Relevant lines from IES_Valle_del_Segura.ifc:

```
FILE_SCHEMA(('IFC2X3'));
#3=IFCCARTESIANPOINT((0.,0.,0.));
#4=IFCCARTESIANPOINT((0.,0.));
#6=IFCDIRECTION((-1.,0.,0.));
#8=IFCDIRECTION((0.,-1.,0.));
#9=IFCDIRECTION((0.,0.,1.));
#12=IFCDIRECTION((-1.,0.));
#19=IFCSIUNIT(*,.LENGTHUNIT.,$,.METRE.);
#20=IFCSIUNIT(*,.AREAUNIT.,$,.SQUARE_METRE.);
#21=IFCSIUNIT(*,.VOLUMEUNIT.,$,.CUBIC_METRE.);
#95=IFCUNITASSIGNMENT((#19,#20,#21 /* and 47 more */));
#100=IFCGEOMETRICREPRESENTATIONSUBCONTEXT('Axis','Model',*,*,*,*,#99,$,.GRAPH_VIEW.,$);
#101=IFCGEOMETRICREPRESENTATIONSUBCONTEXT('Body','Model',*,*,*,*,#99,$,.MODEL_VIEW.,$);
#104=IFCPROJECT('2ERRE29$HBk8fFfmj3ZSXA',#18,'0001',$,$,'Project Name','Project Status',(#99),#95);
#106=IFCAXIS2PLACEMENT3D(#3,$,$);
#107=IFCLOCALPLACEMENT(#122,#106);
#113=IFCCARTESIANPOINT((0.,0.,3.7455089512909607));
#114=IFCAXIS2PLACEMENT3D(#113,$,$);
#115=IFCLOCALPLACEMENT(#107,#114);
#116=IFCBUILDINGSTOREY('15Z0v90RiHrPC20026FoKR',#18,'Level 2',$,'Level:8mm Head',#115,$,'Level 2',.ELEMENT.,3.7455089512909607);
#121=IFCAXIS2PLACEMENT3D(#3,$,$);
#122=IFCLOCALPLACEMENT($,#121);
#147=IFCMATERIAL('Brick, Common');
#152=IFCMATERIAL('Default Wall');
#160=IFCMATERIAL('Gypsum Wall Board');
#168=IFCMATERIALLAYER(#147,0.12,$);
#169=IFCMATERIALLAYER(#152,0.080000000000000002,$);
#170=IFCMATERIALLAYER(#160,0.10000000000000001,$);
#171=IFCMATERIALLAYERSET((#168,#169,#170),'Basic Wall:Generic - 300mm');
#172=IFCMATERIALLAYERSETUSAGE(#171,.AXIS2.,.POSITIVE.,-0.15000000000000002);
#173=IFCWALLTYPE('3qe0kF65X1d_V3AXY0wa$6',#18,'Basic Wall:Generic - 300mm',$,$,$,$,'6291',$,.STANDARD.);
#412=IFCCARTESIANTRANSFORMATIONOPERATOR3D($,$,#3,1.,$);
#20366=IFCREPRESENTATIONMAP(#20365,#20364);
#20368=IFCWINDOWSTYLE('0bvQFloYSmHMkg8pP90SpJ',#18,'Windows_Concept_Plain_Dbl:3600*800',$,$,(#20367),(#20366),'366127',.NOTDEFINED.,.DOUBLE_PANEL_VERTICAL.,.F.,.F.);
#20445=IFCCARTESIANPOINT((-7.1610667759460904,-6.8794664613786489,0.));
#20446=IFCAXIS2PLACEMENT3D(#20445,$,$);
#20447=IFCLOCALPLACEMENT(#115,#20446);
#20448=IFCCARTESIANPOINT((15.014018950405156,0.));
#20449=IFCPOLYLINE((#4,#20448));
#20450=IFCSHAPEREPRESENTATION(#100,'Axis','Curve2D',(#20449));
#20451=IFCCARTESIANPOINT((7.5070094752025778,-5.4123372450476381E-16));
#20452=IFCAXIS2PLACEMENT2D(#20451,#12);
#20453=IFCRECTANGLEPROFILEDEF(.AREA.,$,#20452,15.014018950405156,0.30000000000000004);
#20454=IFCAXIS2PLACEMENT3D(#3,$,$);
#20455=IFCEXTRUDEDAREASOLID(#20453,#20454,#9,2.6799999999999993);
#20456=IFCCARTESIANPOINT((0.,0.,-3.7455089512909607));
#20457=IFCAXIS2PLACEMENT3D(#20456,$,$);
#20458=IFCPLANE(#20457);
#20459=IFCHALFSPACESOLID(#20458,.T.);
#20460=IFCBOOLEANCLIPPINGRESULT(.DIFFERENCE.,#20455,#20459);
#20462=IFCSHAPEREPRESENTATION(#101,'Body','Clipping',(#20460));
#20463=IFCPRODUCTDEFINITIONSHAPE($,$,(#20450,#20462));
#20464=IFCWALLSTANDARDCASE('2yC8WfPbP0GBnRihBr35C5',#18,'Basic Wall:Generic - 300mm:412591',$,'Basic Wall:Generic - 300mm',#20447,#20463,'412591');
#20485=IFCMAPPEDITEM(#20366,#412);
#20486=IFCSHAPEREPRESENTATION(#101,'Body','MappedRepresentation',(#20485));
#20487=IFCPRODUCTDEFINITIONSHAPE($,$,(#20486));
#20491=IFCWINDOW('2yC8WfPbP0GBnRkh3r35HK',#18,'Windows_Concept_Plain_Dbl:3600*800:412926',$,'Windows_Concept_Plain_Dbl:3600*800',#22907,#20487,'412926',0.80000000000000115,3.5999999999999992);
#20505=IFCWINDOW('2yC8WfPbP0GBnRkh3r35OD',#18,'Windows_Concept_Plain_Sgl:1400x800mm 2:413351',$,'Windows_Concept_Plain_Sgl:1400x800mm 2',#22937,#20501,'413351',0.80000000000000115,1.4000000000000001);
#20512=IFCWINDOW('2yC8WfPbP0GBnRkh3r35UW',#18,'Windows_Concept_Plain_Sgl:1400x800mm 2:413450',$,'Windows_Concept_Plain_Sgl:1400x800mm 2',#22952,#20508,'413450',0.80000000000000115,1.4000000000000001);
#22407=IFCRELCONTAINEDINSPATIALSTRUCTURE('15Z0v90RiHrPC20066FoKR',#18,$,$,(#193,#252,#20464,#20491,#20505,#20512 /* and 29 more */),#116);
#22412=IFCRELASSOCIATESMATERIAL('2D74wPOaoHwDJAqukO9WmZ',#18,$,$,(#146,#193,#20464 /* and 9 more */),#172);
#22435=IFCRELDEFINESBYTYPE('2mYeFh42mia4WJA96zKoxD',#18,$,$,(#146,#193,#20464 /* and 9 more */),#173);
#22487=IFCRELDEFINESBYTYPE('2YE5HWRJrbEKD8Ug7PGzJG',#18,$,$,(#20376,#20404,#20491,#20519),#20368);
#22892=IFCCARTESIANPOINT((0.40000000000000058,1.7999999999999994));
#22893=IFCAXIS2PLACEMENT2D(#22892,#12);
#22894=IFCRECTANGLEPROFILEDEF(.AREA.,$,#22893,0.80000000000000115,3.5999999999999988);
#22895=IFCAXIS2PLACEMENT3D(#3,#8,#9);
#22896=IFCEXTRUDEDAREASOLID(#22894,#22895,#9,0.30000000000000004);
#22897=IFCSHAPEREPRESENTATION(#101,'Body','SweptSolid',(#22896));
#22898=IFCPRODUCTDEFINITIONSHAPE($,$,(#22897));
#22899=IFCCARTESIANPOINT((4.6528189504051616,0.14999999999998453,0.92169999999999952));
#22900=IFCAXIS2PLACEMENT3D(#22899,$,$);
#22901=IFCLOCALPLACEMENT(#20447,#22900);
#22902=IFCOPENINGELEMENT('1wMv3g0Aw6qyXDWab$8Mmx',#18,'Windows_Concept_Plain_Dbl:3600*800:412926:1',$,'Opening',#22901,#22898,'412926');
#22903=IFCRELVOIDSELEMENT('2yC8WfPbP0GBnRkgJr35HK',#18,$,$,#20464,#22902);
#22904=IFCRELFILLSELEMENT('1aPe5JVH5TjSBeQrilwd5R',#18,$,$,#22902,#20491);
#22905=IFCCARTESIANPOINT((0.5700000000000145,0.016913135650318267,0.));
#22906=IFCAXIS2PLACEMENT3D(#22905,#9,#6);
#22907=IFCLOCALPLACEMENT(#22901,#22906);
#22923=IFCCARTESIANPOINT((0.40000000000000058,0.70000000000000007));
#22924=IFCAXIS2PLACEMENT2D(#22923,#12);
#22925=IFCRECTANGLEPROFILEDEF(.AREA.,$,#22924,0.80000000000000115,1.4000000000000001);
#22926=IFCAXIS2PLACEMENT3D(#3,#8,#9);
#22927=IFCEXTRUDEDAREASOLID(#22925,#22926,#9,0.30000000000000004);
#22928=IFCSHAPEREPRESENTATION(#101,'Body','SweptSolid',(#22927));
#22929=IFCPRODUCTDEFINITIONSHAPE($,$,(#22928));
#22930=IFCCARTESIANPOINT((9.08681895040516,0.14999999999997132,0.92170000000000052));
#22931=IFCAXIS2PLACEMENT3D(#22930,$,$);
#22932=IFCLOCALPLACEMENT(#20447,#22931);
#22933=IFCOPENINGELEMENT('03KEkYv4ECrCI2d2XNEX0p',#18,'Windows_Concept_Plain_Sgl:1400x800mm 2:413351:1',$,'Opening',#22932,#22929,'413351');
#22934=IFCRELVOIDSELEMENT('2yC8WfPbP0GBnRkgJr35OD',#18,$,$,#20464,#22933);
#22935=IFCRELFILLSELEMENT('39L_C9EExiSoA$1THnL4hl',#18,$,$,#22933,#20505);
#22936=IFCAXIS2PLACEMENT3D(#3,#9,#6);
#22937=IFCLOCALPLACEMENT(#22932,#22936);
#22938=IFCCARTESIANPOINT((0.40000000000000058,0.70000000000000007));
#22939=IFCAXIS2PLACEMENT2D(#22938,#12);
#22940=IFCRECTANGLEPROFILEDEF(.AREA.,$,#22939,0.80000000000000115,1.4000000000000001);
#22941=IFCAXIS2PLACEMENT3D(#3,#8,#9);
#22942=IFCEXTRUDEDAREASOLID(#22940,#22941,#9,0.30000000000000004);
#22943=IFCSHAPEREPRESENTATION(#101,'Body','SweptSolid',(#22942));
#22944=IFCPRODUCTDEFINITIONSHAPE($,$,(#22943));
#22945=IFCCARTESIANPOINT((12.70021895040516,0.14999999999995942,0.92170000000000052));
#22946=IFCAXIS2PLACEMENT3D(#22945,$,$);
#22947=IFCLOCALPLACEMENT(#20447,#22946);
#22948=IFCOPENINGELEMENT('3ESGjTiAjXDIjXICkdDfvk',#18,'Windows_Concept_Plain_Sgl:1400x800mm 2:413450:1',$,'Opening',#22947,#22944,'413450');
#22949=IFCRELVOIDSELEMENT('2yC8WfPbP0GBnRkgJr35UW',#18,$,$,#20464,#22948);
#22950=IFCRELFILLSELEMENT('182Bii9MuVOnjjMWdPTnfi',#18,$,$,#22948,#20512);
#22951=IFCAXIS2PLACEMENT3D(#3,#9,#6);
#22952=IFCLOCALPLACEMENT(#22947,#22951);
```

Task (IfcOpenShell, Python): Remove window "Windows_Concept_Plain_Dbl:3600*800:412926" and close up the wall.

```python
import ifcopenshell
import ifcopenshell.api.feature
import ifcopenshell.api.root
import ifcopenshell.geom
import ifcopenshell.util.shape

model = ifcopenshell.open("IES_Valle_del_Segura.ifc")
settings = ifcopenshell.geom.settings()


def volume(element):
    """Net volume in cubic metres, openings subtracted."""
    shape = ifcopenshell.geom.create_shape(settings, element)
    return ifcopenshell.util.shape.get_volume(shape.geometry)


window = model.by_guid("2yC8WfPbP0GBnRkh3r35HK")
opening = window.FillsVoids[0].RelatingOpeningElement
wall = opening.VoidsElements[0].RelatingBuildingElement
before = volume(wall)

ifcopenshell.api.root.remove_product(model, product=window)
ifcopenshell.api.feature.remove_feature(model, feature=opening)

after = volume(wall)

print(f"wall volume {before:.3f} -> {after:.3f} m3")

model.write("IES_Valle_del_Segura_updated.ifc")
```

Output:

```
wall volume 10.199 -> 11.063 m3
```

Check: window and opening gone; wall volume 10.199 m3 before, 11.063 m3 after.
